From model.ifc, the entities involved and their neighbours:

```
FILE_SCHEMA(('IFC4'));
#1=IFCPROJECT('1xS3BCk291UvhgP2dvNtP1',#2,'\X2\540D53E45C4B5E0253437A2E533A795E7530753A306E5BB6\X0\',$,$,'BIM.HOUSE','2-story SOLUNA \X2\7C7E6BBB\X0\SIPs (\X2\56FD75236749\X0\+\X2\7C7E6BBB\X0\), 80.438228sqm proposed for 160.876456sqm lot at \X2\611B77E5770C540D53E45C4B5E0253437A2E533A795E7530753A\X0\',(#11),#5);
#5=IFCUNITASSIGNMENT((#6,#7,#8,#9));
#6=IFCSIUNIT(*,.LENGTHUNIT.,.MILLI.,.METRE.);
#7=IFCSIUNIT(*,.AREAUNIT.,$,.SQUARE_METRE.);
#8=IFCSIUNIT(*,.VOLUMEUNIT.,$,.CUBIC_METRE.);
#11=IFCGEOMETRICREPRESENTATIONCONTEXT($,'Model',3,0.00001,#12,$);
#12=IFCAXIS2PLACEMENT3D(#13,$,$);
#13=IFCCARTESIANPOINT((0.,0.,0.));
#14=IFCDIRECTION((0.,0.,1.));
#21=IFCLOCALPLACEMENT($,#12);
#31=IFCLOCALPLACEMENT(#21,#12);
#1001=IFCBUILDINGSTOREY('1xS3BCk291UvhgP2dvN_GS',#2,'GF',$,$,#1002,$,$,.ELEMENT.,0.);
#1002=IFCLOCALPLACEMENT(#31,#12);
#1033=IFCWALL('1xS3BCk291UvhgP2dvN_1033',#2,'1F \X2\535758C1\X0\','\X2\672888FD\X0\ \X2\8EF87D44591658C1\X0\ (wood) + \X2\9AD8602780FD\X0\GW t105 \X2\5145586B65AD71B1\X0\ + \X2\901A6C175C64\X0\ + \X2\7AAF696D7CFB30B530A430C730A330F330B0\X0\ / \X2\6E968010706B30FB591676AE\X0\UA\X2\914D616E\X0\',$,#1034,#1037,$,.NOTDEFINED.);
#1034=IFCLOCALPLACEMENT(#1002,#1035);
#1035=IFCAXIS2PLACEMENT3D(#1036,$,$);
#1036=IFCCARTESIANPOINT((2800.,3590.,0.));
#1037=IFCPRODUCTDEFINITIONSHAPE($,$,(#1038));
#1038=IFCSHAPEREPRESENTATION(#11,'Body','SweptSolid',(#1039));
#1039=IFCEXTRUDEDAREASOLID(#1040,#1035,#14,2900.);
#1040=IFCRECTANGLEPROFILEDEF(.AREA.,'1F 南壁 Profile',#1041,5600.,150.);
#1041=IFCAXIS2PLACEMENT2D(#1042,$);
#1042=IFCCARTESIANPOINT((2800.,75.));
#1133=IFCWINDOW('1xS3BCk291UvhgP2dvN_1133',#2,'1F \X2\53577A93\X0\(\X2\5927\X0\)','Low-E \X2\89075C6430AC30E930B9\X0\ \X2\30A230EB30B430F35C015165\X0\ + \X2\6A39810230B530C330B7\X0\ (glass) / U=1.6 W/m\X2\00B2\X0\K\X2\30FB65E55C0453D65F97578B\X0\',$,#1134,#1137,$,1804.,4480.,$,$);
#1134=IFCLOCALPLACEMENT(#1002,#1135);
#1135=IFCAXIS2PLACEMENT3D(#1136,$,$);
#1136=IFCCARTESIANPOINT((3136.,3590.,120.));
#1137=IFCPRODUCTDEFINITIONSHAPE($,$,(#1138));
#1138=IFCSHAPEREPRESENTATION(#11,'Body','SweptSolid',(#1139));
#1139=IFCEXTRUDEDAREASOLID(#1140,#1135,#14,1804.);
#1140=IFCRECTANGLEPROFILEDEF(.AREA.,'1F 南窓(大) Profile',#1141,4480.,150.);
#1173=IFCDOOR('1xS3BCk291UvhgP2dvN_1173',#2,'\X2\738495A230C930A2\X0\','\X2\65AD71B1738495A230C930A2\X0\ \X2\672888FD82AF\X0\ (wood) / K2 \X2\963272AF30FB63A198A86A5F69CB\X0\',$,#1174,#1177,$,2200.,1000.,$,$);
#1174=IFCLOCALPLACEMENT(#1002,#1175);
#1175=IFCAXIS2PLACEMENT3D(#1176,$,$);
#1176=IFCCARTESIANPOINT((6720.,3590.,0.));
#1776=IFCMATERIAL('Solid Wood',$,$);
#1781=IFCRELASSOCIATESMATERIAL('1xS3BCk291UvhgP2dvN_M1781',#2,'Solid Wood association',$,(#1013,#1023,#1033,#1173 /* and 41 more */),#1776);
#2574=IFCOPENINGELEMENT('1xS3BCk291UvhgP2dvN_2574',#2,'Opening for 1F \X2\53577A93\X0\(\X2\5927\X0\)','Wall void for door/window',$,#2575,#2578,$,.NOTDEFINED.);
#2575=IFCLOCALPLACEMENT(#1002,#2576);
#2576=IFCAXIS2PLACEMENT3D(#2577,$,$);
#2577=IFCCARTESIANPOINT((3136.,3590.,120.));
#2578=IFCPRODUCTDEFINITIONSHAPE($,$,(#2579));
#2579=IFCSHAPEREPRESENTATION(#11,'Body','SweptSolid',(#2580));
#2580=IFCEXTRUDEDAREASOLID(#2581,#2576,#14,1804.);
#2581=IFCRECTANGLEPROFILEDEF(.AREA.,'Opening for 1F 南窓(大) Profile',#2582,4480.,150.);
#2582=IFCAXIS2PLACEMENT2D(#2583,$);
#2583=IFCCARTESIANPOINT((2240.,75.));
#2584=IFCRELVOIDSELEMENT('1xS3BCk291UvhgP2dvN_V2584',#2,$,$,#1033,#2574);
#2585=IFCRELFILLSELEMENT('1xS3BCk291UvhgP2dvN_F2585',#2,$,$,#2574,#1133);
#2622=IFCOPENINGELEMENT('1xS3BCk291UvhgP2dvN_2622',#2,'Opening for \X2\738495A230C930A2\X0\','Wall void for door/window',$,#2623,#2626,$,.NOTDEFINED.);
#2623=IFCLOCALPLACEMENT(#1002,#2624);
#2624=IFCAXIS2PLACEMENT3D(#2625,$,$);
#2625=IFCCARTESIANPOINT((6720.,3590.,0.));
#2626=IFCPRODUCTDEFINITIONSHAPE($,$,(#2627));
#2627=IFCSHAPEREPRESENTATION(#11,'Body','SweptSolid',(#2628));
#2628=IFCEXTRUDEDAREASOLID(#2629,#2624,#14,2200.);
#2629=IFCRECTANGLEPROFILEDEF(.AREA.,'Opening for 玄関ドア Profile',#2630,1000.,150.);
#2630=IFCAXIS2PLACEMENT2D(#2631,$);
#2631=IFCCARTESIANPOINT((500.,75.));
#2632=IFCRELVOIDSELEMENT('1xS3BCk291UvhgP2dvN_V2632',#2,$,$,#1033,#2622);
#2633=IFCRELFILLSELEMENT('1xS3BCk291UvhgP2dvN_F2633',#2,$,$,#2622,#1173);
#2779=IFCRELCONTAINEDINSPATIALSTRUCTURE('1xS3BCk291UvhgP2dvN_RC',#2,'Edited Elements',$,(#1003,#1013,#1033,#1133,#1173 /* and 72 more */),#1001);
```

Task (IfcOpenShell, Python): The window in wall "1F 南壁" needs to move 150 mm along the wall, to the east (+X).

```python
import ifcopenshell
import ifcopenshell.api.geometry
import ifcopenshell.util.placement

model = ifcopenshell.open("model.ifc")

window = model.by_guid("1xS3BCk291UvhgP2dvN_1133")
opening = window.FillsVoids[0].RelatingOpeningElement
wall = opening.VoidsElements[0].RelatingBuildingElement

wall_matrix = ifcopenshell.util.placement.get_local_placement(wall.ObjectPlacement)
shift = wall_matrix[:3, 0] * 150.0
before = ifcopenshell.util.placement.get_local_placement(window.ObjectPlacement)[:3, 3].copy()

# The window is not placed relative to its opening, so move both.
for product in (opening, window):
    matrix = ifcopenshell.util.placement.get_local_placement(product.ObjectPlacement)
    matrix[:3, 3] += shift
    ifcopenshell.api.geometry.edit_object_placement(model, product=product, matrix=matrix, is_si=False)

after = ifcopenshell.util.placement.get_local_placement(window.ObjectPlacement)[:3, 3]
print("window moved by", (after - before).round(3) + 0.0)

model.write("model_edited.ifc")
```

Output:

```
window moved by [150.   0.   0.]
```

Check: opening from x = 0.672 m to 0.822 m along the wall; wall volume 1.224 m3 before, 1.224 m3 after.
